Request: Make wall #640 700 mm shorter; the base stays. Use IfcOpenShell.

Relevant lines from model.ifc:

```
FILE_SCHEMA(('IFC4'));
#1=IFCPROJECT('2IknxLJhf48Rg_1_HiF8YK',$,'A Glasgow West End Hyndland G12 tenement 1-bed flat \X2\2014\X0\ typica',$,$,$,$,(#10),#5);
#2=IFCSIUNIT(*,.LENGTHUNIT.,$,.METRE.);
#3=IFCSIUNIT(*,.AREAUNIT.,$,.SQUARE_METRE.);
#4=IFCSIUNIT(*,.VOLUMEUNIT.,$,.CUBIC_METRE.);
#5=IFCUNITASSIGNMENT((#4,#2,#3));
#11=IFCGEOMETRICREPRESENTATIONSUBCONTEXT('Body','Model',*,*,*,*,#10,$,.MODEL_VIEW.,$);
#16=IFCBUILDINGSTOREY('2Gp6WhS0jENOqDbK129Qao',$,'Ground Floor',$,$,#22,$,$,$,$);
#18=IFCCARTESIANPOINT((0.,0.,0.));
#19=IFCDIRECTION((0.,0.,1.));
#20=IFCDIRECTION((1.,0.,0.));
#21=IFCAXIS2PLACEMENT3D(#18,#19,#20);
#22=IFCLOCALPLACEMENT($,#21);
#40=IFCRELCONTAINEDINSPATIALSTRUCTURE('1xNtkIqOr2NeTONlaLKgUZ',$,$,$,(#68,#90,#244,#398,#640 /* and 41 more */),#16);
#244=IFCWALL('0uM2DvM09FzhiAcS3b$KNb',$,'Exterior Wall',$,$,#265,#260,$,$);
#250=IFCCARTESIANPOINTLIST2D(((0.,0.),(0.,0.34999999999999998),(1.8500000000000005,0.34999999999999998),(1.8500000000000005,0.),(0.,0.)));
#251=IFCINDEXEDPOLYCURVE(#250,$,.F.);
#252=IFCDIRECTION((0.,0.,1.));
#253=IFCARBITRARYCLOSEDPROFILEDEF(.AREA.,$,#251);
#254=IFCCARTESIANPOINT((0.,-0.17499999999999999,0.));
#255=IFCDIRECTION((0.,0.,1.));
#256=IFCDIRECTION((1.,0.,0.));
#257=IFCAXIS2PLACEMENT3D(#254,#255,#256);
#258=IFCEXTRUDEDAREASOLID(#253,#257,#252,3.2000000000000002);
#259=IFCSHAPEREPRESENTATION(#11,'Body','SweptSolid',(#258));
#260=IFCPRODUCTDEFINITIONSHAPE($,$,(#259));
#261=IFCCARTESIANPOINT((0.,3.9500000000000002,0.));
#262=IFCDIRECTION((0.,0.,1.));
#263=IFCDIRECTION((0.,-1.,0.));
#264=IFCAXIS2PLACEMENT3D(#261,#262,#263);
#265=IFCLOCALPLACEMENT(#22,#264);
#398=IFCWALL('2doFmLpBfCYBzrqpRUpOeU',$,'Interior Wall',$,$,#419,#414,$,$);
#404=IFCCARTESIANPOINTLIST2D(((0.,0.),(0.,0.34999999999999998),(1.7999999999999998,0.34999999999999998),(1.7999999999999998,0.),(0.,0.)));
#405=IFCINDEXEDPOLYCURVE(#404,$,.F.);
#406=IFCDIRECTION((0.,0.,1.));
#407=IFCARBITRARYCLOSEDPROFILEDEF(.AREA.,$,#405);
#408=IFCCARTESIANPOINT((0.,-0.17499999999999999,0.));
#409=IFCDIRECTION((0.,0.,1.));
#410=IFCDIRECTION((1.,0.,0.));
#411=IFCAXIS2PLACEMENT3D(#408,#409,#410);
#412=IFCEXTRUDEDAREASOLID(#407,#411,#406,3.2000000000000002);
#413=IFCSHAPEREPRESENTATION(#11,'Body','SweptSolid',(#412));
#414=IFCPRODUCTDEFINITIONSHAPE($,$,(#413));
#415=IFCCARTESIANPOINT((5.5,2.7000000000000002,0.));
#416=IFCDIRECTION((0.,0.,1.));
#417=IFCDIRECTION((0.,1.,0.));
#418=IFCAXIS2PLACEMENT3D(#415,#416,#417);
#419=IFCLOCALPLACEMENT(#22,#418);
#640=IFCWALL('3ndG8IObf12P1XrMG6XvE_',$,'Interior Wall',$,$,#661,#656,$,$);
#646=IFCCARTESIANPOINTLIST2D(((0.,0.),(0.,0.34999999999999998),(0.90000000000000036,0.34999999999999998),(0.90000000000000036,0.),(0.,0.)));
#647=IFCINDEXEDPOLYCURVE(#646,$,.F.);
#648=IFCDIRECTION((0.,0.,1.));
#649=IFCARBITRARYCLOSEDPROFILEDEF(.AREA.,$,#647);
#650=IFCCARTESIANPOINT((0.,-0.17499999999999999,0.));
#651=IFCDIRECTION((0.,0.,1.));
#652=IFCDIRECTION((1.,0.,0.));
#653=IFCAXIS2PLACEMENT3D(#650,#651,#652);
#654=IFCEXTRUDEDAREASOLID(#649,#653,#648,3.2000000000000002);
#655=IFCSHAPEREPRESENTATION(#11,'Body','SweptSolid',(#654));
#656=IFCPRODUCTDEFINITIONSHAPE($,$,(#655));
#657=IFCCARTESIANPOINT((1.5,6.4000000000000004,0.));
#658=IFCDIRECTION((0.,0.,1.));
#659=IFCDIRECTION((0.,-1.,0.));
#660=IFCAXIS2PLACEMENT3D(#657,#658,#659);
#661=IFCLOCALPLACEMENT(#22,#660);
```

```python
import ifcopenshell
import ifcopenshell.geom
import ifcopenshell.util.representation
import ifcopenshell.util.shape

model = ifcopenshell.open("model.ifc")
settings = ifcopenshell.geom.settings()


def volume(element):
    """Net volume in cubic metres, openings subtracted."""
    shape = ifcopenshell.geom.create_shape(settings, element)
    return ifcopenshell.util.shape.get_volume(shape.geometry)


wall = model.by_id(640)
before = volume(wall)

body = ifcopenshell.util.representation.get_representation(wall, "Model", "Body")
solid = body.Items[0]
old_height = solid.Depth
solid.Depth -= 0.7
after = volume(wall)

print(f"height {old_height:g} -> {solid.Depth:g}, volume {before:.3f} -> {after:.3f} m3")

model.write("model_updated.ifc")
```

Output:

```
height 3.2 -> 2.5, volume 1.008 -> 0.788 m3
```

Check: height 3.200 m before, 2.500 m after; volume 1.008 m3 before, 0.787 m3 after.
